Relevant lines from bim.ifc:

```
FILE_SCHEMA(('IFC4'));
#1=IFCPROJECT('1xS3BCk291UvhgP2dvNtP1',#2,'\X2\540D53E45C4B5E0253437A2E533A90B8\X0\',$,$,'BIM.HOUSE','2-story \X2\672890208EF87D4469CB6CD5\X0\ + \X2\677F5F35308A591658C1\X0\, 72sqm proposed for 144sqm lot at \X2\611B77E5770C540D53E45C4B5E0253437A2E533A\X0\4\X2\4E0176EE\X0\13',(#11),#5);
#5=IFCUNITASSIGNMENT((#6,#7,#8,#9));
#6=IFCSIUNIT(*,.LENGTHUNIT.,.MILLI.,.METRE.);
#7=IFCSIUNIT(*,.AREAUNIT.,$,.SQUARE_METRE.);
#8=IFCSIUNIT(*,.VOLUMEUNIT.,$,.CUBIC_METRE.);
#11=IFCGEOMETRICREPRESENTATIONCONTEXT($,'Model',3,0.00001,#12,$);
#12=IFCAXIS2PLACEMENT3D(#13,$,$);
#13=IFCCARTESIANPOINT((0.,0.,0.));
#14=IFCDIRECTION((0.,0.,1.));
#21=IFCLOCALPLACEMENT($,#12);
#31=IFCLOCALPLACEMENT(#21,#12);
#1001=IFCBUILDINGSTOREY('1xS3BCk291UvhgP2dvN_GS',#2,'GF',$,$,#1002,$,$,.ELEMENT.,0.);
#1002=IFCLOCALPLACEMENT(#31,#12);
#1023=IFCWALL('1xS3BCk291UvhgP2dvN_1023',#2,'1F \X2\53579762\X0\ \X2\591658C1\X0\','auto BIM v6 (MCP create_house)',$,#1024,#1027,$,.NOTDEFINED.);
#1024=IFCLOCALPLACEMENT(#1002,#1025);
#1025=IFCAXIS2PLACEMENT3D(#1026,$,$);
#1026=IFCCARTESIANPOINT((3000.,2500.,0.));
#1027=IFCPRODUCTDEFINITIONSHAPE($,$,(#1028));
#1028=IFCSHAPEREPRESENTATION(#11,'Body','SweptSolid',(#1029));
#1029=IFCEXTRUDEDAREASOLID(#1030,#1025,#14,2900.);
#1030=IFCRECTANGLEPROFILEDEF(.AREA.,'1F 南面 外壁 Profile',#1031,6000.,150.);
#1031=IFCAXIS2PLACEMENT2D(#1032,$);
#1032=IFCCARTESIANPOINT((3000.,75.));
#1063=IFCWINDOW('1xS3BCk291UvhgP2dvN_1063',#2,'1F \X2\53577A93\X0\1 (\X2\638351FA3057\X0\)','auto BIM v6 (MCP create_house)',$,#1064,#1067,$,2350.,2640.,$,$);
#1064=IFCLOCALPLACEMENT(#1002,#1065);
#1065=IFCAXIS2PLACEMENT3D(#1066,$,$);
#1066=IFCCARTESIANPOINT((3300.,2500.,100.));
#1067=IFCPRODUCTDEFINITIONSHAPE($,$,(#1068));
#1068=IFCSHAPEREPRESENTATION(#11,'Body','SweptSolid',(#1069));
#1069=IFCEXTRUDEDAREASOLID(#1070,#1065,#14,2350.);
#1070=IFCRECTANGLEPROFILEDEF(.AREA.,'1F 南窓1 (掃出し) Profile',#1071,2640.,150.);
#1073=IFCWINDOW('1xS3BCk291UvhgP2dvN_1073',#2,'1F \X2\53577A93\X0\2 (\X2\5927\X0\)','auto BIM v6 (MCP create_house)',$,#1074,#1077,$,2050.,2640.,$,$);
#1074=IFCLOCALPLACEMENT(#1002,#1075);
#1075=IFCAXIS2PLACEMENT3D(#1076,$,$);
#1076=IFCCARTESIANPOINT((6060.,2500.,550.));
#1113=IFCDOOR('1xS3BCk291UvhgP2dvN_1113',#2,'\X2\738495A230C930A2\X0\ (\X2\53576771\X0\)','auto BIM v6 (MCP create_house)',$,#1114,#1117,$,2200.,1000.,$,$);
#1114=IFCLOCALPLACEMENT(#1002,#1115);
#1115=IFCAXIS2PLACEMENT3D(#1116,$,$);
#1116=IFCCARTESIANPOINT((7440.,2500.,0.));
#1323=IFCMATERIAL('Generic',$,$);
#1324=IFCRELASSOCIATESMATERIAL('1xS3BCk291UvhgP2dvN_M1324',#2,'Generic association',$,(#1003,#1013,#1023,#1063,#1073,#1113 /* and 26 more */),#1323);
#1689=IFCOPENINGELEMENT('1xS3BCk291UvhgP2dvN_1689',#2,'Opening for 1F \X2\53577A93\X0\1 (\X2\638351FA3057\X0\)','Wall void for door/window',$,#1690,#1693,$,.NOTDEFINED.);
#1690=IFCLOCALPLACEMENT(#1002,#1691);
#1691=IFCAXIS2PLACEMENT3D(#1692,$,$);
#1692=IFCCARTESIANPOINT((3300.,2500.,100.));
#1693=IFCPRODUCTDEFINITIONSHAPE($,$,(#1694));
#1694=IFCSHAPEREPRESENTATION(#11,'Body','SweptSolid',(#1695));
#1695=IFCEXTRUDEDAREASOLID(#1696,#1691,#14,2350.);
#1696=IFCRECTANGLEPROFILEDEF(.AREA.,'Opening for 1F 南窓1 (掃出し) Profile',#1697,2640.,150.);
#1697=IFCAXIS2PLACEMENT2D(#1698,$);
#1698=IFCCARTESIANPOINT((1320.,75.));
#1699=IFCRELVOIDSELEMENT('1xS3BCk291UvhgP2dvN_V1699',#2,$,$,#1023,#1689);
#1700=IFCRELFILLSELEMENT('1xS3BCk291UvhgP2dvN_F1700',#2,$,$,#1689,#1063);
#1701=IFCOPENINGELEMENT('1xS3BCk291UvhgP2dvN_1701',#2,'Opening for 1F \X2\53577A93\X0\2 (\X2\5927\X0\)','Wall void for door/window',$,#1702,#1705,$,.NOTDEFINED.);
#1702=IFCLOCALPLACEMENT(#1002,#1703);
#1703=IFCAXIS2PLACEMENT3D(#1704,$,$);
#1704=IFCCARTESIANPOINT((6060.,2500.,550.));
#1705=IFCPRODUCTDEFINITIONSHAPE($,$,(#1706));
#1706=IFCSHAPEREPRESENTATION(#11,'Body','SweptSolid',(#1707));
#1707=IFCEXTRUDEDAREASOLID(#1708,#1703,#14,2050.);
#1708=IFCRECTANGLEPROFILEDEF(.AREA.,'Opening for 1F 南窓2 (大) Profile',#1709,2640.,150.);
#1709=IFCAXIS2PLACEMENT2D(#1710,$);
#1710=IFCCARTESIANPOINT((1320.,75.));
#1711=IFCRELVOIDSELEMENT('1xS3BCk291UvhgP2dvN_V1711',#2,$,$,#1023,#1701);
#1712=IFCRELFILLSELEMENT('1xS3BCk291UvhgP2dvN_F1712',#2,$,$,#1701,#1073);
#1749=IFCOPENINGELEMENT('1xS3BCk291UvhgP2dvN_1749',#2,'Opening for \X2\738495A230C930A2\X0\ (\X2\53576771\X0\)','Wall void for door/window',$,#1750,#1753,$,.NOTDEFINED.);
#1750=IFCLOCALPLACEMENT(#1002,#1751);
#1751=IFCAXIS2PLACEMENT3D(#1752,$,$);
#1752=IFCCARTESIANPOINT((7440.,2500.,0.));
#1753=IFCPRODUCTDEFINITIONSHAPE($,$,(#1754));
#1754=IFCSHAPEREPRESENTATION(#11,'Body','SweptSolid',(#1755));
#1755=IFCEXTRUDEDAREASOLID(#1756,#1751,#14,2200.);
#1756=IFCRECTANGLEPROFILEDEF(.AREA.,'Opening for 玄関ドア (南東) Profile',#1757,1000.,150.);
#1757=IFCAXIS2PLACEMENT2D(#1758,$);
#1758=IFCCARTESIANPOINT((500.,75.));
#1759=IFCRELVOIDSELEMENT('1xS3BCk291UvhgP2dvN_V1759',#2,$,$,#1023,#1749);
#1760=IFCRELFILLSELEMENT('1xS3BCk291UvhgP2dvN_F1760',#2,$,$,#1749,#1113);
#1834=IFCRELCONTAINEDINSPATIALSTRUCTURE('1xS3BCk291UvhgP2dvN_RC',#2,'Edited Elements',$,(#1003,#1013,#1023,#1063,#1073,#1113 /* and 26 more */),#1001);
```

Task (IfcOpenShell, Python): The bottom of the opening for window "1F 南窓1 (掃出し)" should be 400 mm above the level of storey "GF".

```python
import numpy as np
import ifcopenshell
import ifcopenshell.api.geometry
import ifcopenshell.geom
import ifcopenshell.util.element
import ifcopenshell.util.placement
import ifcopenshell.util.shape
import ifcopenshell.util.unit

model = ifcopenshell.open("bim.ifc")
unit_scale = ifcopenshell.util.unit.calculate_unit_scale(model)

window = model.by_id(1063)
opening = window.FillsVoids[0].RelatingOpeningElement
storey = ifcopenshell.util.element.get_container(window, ifc_class="IfcBuildingStorey")
level = ifcopenshell.util.placement.get_local_placement(storey.ObjectPlacement)[2, 3]

# The opening's origin need not be at the sill, so measure its lowest point.
shape = ifcopenshell.geom.create_shape(ifcopenshell.geom.settings(), opening)
bottom = ifcopenshell.util.shape.get_shape_bottom_elevation(shape, shape.geometry) / unit_scale
dz = level + 0.4 / unit_scale - bottom

shift = np.array([0.0, 0.0, dz])
# The window is not placed relative to its opening, so move both.
for product in (opening, window):
    matrix = ifcopenshell.util.placement.get_local_placement(product.ObjectPlacement)
    matrix[:3, 3] += shift
    ifcopenshell.api.geometry.edit_object_placement(model, product=product, matrix=matrix, is_si=False)

print(f"moved by {dz * unit_scale:+.3f} m")

model.write("bim_rev.ifc")
```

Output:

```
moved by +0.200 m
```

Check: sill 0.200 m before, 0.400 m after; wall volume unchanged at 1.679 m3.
